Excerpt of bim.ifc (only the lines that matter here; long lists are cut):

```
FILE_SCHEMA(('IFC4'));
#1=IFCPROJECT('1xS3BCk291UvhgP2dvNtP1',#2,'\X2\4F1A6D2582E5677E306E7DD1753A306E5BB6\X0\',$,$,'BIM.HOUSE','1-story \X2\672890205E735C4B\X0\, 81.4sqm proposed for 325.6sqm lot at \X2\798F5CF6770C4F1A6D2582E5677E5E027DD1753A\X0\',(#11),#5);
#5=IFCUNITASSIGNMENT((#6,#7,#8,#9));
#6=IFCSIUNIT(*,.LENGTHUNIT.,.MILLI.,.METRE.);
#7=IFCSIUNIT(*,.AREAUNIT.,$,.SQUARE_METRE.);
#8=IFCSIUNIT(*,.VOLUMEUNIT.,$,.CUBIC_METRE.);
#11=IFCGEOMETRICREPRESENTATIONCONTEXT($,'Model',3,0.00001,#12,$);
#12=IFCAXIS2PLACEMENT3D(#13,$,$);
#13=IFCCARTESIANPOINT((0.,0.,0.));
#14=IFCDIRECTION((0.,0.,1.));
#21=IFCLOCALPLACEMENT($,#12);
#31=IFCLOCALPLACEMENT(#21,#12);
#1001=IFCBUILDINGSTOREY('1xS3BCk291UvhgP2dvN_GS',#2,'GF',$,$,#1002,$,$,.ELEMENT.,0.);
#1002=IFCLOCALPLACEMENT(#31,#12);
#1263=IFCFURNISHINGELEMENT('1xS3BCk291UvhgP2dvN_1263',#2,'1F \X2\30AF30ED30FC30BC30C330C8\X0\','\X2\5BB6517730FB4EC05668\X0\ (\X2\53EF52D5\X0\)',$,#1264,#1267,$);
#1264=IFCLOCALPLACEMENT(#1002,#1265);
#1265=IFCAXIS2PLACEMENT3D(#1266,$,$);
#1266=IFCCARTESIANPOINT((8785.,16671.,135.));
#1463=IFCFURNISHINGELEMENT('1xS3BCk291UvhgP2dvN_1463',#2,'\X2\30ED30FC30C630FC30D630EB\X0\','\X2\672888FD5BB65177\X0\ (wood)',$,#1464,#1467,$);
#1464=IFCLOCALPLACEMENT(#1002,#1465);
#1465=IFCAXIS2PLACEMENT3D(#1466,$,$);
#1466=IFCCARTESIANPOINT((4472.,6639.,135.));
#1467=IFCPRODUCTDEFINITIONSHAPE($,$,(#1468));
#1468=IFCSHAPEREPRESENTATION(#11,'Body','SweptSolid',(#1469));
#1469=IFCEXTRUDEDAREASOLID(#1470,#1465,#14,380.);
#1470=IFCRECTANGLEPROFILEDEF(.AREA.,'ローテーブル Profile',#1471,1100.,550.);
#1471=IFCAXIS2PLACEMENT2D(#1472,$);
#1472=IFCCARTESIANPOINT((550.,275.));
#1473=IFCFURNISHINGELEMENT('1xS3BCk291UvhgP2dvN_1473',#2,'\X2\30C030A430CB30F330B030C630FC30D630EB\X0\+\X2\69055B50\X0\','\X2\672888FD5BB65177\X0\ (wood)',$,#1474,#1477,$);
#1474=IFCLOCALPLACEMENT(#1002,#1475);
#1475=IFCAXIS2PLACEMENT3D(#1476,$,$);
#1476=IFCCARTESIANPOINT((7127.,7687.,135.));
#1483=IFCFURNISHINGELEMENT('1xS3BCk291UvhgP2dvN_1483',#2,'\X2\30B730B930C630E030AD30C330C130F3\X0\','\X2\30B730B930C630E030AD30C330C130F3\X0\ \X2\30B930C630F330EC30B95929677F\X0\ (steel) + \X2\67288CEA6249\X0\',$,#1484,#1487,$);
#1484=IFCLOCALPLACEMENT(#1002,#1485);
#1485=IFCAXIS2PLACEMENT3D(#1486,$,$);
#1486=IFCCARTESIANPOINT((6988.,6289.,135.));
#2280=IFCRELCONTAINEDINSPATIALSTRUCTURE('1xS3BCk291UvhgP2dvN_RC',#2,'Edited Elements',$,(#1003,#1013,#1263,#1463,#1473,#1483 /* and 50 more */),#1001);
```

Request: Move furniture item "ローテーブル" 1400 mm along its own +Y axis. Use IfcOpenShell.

```python
import ifcopenshell
import ifcopenshell.api.geometry
import ifcopenshell.util.placement

model = ifcopenshell.open("bim.ifc")

item = model.by_id(1463)
matrix = ifcopenshell.util.placement.get_local_placement(item.ObjectPlacement)
matrix[:3, 3] += matrix[:3, 1] * 1400.0
ifcopenshell.api.geometry.edit_object_placement(model, product=item, matrix=matrix, is_si=False)

print(ifcopenshell.util.placement.get_local_placement(item.ObjectPlacement).round(3) + 0.0)

model.write("bim_updated.ifc")
```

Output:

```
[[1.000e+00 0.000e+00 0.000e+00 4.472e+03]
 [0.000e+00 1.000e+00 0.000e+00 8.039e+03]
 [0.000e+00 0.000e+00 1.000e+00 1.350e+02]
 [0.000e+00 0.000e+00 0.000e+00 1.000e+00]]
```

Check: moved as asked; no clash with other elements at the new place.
